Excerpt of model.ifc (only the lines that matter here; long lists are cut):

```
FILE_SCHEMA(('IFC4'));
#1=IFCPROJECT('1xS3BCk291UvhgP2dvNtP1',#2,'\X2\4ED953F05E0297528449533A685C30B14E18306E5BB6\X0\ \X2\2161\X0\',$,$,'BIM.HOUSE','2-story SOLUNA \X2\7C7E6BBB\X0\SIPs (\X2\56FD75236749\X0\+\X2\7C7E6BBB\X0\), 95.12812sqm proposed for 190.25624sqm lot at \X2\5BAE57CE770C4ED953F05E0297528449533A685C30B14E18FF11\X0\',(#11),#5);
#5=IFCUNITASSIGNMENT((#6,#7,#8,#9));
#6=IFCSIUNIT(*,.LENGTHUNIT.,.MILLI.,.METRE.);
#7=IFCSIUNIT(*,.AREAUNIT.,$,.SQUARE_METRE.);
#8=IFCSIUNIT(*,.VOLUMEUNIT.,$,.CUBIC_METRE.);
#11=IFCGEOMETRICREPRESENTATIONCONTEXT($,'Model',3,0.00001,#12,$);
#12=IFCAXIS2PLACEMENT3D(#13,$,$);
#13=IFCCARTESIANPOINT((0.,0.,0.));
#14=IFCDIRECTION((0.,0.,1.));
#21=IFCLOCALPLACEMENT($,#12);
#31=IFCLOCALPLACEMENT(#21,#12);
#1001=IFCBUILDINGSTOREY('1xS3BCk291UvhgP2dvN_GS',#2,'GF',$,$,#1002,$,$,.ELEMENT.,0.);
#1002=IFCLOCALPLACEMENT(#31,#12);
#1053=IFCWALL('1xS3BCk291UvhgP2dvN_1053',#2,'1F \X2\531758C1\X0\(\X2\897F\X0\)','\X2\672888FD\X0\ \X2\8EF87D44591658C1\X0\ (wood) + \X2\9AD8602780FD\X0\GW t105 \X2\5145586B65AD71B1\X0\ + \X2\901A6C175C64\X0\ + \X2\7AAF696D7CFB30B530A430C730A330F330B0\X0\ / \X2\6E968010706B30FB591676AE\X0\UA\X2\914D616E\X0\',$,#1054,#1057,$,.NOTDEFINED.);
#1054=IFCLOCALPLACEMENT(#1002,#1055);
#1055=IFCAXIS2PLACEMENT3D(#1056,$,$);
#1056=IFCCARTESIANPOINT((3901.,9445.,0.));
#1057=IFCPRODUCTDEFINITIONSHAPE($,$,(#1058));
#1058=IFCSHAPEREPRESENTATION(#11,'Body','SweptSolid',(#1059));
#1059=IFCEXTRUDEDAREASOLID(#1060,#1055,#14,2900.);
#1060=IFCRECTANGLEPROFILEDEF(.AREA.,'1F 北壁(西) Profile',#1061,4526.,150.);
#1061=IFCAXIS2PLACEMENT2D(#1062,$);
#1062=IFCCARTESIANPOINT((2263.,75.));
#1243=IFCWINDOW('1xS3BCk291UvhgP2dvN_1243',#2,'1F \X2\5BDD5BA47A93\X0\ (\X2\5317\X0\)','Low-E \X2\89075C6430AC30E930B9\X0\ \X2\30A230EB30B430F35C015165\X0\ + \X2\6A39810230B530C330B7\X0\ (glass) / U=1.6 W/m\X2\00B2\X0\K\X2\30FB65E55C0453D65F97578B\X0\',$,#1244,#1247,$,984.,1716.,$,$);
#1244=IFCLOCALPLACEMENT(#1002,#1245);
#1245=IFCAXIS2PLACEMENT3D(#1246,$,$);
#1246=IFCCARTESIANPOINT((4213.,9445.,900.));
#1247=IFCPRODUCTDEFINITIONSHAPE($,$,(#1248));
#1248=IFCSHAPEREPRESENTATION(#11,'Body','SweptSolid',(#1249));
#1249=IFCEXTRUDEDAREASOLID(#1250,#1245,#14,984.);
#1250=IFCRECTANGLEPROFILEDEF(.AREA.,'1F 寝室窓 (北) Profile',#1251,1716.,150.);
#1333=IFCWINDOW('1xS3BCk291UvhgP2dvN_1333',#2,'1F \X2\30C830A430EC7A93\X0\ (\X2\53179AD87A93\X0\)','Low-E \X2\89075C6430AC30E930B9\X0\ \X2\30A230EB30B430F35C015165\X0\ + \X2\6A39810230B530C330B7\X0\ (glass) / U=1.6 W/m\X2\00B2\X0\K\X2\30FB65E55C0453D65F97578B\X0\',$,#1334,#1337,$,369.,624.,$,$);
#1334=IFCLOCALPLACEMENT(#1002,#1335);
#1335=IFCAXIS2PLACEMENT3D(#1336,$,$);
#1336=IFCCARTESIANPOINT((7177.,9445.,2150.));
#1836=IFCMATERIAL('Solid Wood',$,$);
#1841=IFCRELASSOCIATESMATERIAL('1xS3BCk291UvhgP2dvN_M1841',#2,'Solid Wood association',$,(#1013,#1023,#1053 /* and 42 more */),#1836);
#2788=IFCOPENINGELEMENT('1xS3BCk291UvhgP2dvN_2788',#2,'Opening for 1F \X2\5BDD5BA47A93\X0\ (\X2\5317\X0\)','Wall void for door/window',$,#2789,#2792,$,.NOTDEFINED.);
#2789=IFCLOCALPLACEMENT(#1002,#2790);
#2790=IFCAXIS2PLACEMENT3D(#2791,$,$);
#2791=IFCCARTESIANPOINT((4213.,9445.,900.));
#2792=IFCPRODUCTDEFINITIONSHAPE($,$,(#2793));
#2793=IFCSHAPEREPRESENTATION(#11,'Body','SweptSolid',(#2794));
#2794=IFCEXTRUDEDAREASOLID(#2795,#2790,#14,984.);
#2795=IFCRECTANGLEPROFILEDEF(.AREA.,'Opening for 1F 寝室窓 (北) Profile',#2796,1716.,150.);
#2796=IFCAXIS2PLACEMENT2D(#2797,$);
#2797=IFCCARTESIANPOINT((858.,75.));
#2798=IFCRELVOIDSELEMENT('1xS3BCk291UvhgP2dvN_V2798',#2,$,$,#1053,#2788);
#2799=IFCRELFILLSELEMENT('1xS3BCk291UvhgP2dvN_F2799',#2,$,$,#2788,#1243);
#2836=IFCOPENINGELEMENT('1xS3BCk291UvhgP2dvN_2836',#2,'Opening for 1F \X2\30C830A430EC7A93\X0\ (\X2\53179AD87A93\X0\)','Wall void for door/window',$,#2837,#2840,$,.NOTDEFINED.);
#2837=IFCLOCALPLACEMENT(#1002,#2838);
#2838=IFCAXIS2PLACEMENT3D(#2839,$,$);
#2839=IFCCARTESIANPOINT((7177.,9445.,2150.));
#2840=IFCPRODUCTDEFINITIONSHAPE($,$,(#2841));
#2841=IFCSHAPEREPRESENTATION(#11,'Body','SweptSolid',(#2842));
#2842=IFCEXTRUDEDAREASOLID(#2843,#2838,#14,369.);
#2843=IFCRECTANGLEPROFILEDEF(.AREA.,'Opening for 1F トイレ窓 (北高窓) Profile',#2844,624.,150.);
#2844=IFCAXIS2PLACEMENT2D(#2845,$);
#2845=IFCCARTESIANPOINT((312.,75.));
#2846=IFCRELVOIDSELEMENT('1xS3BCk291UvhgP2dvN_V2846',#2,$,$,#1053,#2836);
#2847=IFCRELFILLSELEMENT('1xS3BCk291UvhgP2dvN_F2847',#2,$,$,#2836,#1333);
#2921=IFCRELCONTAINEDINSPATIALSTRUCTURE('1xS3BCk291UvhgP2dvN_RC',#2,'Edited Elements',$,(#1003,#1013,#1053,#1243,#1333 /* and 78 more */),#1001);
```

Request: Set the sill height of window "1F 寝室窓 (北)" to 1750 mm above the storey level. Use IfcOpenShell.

```python
import numpy as np
import ifcopenshell
import ifcopenshell.api.geometry
import ifcopenshell.geom
import ifcopenshell.util.element
import ifcopenshell.util.placement
import ifcopenshell.util.shape
import ifcopenshell.util.unit

model = ifcopenshell.open("model.ifc")
unit_scale = ifcopenshell.util.unit.calculate_unit_scale(model)

window = model.by_guid("1xS3BCk291UvhgP2dvN_1243")
opening = window.FillsVoids[0].RelatingOpeningElement
storey = ifcopenshell.util.element.get_container(window, ifc_class="IfcBuildingStorey")
level = ifcopenshell.util.placement.get_local_placement(storey.ObjectPlacement)[2, 3]

# The opening's origin need not be at the sill, so measure its lowest point.
shape = ifcopenshell.geom.create_shape(ifcopenshell.geom.settings(), opening)
bottom = ifcopenshell.util.shape.get_shape_bottom_elevation(shape, shape.geometry) / unit_scale
dz = level + 1750.0 - bottom

shift = np.array([0.0, 0.0, dz])
# The window is not placed relative to its opening, so move both.
for product in (opening, window):
    matrix = ifcopenshell.util.placement.get_local_placement(product.ObjectPlacement)
    matrix[:3, 3] += shift
    ifcopenshell.api.geometry.edit_object_placement(model, product=product, matrix=matrix, is_si=False)

print(f"moved by {dz * unit_scale:+.3f} m")

model.write("model-out.ifc")
```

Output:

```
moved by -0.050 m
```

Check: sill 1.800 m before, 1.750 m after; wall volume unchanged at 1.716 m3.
